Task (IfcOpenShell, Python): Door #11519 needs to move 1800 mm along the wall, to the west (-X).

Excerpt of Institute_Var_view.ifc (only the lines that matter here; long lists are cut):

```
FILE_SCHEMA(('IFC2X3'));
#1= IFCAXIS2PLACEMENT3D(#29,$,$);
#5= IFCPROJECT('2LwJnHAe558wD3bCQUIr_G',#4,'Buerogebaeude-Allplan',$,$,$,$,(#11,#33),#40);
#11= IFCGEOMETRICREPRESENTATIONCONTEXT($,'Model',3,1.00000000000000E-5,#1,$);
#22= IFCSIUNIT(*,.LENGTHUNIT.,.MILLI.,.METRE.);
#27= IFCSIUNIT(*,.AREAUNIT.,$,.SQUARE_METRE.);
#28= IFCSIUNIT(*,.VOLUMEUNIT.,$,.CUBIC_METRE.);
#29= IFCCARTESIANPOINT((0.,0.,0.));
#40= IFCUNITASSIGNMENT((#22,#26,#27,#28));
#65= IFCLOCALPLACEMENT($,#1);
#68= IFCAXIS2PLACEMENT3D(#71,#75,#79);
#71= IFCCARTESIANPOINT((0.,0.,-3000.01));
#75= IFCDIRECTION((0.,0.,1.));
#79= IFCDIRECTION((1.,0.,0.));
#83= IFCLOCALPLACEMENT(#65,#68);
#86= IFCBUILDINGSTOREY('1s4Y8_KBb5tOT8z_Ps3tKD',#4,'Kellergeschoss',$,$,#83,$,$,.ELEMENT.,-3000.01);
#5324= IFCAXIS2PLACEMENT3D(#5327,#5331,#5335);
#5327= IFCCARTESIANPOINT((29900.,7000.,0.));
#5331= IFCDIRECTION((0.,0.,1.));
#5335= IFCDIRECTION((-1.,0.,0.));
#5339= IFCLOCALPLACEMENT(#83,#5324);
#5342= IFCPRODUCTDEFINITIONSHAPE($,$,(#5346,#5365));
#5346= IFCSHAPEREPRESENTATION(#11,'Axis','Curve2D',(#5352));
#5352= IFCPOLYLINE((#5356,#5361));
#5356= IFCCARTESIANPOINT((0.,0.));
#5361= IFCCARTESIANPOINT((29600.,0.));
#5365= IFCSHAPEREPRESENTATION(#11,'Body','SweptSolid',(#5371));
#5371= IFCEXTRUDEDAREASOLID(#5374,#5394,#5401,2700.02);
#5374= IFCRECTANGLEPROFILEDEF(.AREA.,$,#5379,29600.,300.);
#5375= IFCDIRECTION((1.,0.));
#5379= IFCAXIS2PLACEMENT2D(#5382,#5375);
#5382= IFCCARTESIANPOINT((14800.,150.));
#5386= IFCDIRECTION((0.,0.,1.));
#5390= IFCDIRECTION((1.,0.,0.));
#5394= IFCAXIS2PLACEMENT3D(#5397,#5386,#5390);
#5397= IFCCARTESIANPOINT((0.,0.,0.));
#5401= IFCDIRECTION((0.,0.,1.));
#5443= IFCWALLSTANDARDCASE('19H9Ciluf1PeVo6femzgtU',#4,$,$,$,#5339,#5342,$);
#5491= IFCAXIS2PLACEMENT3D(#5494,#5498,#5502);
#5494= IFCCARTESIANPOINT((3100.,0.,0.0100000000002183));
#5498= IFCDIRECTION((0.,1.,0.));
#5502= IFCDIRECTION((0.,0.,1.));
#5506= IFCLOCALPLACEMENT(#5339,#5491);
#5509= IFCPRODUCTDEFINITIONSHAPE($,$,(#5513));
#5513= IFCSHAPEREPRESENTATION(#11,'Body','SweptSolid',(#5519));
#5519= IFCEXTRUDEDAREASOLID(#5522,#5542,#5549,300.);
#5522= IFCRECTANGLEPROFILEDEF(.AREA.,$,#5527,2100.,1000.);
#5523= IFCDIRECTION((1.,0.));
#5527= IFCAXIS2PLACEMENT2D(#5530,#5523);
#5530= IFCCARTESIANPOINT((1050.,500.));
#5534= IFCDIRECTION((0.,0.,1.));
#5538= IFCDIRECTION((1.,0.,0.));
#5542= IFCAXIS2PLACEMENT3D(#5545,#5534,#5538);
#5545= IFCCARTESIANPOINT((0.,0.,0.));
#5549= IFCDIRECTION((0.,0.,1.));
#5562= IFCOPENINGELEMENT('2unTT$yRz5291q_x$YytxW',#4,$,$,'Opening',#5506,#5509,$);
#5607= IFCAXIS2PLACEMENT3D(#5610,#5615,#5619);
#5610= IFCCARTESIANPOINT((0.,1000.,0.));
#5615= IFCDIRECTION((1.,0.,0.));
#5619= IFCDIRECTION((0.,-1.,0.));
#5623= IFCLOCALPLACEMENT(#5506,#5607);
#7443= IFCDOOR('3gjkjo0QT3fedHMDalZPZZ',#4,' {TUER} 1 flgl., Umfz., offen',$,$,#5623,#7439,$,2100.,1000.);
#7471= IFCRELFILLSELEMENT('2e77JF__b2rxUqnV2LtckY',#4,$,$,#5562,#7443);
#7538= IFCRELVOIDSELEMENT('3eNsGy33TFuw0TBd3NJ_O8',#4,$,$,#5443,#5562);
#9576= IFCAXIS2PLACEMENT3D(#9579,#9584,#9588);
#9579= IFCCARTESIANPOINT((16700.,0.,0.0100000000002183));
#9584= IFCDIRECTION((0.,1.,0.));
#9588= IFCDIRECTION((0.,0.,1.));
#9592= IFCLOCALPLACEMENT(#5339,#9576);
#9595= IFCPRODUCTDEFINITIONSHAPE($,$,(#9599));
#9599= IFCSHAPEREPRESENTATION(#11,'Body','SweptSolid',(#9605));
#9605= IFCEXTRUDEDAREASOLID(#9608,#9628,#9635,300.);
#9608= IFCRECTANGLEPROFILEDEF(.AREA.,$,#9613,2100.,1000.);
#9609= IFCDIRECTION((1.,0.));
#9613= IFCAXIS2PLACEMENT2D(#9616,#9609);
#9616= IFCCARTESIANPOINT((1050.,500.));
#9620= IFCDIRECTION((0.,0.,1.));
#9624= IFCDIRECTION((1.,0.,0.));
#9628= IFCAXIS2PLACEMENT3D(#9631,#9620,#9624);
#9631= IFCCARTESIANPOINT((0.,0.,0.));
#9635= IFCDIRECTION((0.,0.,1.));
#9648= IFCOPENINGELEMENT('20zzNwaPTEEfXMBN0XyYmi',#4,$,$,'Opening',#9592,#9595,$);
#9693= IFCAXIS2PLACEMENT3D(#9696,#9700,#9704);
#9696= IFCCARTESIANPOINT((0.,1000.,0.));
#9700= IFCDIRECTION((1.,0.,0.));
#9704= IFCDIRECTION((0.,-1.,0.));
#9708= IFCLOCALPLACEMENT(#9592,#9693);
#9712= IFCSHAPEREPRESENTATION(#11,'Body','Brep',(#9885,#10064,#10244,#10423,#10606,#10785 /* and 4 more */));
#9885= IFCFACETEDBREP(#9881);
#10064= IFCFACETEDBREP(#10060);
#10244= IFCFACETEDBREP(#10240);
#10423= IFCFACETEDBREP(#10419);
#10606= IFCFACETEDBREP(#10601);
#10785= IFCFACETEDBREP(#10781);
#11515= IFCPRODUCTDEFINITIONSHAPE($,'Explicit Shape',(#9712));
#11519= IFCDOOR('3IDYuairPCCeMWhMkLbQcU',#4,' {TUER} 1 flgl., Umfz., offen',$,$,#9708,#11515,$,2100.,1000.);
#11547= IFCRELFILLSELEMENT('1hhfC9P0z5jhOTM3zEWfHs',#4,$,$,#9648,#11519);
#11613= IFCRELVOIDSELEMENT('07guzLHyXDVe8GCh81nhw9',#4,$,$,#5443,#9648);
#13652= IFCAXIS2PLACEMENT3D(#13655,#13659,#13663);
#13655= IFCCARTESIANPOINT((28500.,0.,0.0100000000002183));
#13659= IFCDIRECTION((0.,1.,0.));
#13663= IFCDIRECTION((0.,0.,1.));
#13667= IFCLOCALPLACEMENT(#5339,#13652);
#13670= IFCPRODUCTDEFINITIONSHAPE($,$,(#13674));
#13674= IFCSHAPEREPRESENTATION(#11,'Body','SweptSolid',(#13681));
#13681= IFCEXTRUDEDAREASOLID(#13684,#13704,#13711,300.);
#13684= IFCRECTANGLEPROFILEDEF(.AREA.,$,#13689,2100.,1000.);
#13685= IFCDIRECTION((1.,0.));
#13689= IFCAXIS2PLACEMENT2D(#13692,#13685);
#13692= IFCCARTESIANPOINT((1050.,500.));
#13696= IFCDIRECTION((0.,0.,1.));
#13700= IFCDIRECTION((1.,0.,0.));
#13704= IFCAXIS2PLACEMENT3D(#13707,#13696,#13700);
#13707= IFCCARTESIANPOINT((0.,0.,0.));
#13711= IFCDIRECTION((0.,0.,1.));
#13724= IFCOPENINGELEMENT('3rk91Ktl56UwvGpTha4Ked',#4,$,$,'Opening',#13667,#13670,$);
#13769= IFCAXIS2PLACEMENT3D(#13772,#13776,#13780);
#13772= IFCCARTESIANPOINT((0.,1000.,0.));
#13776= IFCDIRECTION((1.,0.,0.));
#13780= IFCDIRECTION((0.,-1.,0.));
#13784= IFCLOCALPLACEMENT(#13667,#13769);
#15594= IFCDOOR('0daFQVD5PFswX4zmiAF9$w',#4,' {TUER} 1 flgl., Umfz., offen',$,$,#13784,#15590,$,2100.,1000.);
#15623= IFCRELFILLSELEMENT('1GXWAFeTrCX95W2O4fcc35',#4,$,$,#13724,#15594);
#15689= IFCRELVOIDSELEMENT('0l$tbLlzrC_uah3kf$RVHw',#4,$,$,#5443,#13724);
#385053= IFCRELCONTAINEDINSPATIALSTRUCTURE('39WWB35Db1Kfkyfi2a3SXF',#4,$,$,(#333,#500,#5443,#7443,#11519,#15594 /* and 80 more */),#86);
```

```python
import ifcopenshell
import ifcopenshell.api.geometry
import ifcopenshell.util.placement
import ifcopenshell.util.unit

model = ifcopenshell.open("Institute_Var_view.ifc")
unit_scale = ifcopenshell.util.unit.calculate_unit_scale(model)

door = model.by_guid("3IDYuairPCCeMWhMkLbQcU")
opening = door.FillsVoids[0].RelatingOpeningElement
wall = opening.VoidsElements[0].RelatingBuildingElement

wall_matrix = ifcopenshell.util.placement.get_local_placement(wall.ObjectPlacement)
shift = wall_matrix[:3, 0] * 1.8 / unit_scale
before = ifcopenshell.util.placement.get_local_placement(door.ObjectPlacement)[:3, 3].copy()

# The door is placed relative to its opening, so it follows when the opening moves.
matrix = ifcopenshell.util.placement.get_local_placement(opening.ObjectPlacement)
matrix[:3, 3] += shift
ifcopenshell.api.geometry.edit_object_placement(
    model, product=opening, matrix=matrix, is_si=False, should_transform_children=True
)

after = ifcopenshell.util.placement.get_local_placement(door.ObjectPlacement)[:3, 3]
print("door moved by", (after - before).round(3) + 0.0)

model.write("Institute_Var_view_updated.ifc")
```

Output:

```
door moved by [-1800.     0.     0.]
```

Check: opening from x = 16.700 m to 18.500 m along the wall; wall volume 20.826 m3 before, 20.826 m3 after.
